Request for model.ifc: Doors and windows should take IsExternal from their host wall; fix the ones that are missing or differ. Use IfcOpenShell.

First a look at what the model holds.

```python
import ifcopenshell
import ifcopenshell.util.element

model = ifcopenshell.open("model.ifc")
print(model.schema)
seen = {}
for e in model.by_type("IfcDoor") + model.by_type("IfcWindow"):
    if not e.FillsVoids:
        continue
    host = e.FillsVoids[0].RelatingOpeningElement.VoidsElements[0].RelatingBuildingElement
    own = ifcopenshell.util.element.get_pset(e, f"Pset_{e.is_a()[3:].removesuffix('StandardCase')}Common", "IsExternal")
    wall = ifcopenshell.util.element.get_pset(host, "Pset_WallCommon", "IsExternal")
    seen[e.is_a(), own, wall] = seen.get((e.is_a(), own, wall), 0) + 1
for (cls, own, wall), count in sorted(seen.items(), key=str):
    print(count, cls, "IsExternal:", own, "| host wall:", wall)
```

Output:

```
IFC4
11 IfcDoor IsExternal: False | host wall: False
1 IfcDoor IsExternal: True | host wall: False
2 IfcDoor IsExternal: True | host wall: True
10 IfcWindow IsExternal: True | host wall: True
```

```python
import ifcopenshell
import ifcopenshell.api.pset
import ifcopenshell.util.element

model = ifcopenshell.open("model.ifc")

count = 0
for ifc_class, pset_name in (("IfcDoor", "Pset_DoorCommon"), ("IfcWindow", "Pset_WindowCommon")):
    for e in model.by_type(ifc_class):
        if not e.FillsVoids:
            continue
        host = e.FillsVoids[0].RelatingOpeningElement.VoidsElements[0].RelatingBuildingElement
        external = ifcopenshell.util.element.get_pset(host, "Pset_WallCommon", "IsExternal")
        if external is None or ifcopenshell.util.element.get_pset(e, pset_name, "IsExternal") == external:
            continue
        pset = ifcopenshell.api.pset.add_pset(model, product=e, name=pset_name)
        ifcopenshell.api.pset.edit_pset(model, pset=pset, properties={"IsExternal": external})
        count += 1

print(count, "updated")

model.write("model_rev.ifc")
```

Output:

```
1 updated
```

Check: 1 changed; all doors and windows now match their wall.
